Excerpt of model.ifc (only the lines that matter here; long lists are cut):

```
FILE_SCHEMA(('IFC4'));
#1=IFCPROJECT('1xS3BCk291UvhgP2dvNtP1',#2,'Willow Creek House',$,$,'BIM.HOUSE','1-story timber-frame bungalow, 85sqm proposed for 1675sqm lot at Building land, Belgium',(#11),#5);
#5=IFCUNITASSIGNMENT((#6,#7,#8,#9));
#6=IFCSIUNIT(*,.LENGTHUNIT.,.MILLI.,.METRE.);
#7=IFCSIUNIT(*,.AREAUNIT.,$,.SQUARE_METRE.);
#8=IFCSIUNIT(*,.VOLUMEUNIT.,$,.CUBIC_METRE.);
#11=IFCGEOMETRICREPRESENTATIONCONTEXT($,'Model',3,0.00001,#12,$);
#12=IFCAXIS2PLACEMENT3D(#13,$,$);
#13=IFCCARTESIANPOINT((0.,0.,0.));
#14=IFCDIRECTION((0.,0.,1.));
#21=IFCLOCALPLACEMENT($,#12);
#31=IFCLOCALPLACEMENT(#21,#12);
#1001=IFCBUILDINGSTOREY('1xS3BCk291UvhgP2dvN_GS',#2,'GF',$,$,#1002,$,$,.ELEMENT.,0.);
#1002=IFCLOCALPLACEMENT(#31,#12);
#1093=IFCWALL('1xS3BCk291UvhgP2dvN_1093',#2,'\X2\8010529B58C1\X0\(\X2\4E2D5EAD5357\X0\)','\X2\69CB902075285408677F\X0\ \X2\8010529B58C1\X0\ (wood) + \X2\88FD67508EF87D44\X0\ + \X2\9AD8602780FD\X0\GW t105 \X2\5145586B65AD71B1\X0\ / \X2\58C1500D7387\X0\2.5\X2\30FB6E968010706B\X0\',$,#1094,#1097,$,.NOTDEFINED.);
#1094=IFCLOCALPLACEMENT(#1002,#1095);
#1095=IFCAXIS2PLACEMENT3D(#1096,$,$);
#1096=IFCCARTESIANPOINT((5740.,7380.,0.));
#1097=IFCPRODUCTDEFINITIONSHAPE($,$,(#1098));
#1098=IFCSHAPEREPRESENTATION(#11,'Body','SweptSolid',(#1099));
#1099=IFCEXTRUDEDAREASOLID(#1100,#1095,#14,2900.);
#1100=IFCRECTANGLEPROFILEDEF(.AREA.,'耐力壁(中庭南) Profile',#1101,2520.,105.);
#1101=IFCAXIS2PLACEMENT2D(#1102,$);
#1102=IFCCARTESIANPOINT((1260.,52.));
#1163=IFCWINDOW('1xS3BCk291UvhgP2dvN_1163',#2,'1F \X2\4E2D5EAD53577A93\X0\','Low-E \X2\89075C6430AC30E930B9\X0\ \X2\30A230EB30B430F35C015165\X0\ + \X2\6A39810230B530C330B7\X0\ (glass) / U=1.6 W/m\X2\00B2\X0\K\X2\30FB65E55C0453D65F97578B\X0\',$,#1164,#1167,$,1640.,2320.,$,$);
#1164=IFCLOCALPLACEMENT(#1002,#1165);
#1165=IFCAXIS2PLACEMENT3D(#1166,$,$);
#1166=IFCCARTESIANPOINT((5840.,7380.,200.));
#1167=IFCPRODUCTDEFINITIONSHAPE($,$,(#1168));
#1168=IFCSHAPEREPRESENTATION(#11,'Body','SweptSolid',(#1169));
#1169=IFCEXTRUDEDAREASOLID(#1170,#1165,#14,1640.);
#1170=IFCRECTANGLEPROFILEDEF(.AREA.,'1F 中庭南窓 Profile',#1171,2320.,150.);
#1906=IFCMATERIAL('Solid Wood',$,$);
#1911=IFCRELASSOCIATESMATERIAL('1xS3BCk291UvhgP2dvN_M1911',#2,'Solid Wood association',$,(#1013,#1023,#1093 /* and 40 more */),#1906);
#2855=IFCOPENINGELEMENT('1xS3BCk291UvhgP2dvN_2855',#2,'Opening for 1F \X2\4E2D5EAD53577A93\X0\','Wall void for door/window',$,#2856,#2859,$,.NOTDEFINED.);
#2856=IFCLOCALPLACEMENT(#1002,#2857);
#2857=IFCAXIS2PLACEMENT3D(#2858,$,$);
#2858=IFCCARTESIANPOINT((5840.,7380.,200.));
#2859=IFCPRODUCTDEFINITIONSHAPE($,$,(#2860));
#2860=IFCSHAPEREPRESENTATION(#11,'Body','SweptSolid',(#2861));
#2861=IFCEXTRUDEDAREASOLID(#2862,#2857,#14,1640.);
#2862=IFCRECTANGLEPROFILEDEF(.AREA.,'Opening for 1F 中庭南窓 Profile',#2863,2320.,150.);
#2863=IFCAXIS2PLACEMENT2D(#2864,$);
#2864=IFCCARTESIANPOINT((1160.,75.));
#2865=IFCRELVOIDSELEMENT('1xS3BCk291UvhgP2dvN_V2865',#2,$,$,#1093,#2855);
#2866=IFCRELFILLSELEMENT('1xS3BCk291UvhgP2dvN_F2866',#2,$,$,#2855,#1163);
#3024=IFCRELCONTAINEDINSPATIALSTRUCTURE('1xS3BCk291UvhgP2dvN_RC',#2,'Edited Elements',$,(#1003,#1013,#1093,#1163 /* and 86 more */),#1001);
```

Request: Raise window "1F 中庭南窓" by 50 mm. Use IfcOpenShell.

```python
import numpy as np
import ifcopenshell
import ifcopenshell.api.geometry
import ifcopenshell.util.placement
import ifcopenshell.util.unit

model = ifcopenshell.open("model.ifc")
unit_scale = ifcopenshell.util.unit.calculate_unit_scale(model)

window = model.by_id(1163)
opening = window.FillsVoids[0].RelatingOpeningElement
dz = 50.0

shift = np.array([0.0, 0.0, dz])
# The window is not placed relative to its opening, so move both.
for product in (opening, window):
    matrix = ifcopenshell.util.placement.get_local_placement(product.ObjectPlacement)
    matrix[:3, 3] += shift
    ifcopenshell.api.geometry.edit_object_placement(model, product=product, matrix=matrix, is_si=False)

print(f"moved by {dz * unit_scale:+.3f} m")

model.write("model-out.ifc")
```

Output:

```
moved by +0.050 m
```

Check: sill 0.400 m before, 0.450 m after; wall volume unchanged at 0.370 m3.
